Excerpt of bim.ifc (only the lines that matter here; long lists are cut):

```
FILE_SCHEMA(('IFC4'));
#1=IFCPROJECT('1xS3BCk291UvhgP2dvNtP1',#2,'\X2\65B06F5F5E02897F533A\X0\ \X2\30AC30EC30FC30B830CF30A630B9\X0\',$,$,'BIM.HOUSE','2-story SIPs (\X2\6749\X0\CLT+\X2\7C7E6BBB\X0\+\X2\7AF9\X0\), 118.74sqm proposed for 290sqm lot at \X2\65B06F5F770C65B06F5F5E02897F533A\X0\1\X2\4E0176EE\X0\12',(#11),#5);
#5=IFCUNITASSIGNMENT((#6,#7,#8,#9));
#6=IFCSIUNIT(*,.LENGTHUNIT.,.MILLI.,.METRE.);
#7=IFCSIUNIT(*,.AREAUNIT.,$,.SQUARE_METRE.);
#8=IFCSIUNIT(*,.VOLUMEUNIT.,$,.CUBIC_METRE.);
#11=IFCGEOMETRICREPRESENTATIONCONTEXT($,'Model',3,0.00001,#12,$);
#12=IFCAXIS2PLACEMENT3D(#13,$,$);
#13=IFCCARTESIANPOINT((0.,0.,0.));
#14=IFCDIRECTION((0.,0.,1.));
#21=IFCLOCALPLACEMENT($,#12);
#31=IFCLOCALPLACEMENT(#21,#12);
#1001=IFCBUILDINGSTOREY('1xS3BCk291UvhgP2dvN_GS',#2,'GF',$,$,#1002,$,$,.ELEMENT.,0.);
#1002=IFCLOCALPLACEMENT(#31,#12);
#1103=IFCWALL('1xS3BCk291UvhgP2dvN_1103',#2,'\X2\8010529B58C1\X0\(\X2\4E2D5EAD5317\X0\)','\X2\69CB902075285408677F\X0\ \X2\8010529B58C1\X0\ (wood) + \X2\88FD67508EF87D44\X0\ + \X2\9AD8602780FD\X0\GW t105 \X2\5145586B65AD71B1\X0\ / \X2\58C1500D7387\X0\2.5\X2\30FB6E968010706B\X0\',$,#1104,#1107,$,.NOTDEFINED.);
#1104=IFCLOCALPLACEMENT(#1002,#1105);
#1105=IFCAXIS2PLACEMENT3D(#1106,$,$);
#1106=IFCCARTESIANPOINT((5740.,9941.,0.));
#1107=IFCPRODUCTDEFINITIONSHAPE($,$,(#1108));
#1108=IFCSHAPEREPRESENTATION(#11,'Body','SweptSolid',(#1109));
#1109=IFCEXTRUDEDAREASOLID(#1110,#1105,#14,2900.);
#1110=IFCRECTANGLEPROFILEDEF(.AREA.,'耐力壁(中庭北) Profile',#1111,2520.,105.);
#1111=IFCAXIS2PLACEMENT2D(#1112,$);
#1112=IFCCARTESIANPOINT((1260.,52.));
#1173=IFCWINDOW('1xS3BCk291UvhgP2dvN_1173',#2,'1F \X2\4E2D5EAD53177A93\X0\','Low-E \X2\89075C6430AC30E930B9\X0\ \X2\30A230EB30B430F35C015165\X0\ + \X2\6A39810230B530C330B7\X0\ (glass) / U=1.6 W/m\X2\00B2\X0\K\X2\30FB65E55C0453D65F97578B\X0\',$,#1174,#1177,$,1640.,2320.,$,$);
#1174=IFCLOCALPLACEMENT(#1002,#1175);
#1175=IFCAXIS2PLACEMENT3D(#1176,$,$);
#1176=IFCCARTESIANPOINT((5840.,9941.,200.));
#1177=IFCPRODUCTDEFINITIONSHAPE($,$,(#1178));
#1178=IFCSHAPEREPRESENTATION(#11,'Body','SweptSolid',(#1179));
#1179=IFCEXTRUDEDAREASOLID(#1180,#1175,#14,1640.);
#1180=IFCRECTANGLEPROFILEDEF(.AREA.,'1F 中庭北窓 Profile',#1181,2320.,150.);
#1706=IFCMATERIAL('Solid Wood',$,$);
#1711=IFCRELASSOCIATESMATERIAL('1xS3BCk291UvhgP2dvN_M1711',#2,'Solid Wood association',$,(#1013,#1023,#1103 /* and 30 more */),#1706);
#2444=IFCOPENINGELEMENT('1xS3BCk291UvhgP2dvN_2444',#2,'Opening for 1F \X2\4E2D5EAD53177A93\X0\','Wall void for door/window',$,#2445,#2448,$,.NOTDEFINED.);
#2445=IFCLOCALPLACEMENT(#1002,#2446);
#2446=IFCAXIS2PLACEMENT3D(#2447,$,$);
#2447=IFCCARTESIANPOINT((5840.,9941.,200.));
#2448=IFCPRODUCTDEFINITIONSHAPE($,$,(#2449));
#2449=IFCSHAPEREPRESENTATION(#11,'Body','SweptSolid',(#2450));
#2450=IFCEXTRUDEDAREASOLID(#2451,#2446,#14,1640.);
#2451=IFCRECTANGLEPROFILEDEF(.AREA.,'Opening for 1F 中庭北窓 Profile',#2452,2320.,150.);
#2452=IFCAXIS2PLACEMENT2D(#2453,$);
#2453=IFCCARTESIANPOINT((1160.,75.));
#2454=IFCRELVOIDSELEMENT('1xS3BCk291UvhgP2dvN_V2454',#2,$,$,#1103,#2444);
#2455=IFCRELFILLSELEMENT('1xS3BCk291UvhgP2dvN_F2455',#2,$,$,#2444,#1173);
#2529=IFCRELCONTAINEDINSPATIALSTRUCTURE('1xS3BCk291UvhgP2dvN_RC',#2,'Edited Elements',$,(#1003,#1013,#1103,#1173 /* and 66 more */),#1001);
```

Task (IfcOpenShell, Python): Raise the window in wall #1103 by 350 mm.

```python
import numpy as np
import ifcopenshell
import ifcopenshell.api.geometry
import ifcopenshell.util.placement
import ifcopenshell.util.unit

model = ifcopenshell.open("bim.ifc")
unit_scale = ifcopenshell.util.unit.calculate_unit_scale(model)

window = model.by_guid("1xS3BCk291UvhgP2dvN_1173")
opening = window.FillsVoids[0].RelatingOpeningElement
dz = 0.35 / unit_scale

shift = np.array([0.0, 0.0, dz])
# The window is not placed relative to its opening, so move both.
for product in (opening, window):
    matrix = ifcopenshell.util.placement.get_local_placement(product.ObjectPlacement)
    matrix[:3, 3] += shift
    ifcopenshell.api.geometry.edit_object_placement(model, product=product, matrix=matrix, is_si=False)

print(f"moved by {dz * unit_scale:+.3f} m")

model.write("bim_rev.ifc")
```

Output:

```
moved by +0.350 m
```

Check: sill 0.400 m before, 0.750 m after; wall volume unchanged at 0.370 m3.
